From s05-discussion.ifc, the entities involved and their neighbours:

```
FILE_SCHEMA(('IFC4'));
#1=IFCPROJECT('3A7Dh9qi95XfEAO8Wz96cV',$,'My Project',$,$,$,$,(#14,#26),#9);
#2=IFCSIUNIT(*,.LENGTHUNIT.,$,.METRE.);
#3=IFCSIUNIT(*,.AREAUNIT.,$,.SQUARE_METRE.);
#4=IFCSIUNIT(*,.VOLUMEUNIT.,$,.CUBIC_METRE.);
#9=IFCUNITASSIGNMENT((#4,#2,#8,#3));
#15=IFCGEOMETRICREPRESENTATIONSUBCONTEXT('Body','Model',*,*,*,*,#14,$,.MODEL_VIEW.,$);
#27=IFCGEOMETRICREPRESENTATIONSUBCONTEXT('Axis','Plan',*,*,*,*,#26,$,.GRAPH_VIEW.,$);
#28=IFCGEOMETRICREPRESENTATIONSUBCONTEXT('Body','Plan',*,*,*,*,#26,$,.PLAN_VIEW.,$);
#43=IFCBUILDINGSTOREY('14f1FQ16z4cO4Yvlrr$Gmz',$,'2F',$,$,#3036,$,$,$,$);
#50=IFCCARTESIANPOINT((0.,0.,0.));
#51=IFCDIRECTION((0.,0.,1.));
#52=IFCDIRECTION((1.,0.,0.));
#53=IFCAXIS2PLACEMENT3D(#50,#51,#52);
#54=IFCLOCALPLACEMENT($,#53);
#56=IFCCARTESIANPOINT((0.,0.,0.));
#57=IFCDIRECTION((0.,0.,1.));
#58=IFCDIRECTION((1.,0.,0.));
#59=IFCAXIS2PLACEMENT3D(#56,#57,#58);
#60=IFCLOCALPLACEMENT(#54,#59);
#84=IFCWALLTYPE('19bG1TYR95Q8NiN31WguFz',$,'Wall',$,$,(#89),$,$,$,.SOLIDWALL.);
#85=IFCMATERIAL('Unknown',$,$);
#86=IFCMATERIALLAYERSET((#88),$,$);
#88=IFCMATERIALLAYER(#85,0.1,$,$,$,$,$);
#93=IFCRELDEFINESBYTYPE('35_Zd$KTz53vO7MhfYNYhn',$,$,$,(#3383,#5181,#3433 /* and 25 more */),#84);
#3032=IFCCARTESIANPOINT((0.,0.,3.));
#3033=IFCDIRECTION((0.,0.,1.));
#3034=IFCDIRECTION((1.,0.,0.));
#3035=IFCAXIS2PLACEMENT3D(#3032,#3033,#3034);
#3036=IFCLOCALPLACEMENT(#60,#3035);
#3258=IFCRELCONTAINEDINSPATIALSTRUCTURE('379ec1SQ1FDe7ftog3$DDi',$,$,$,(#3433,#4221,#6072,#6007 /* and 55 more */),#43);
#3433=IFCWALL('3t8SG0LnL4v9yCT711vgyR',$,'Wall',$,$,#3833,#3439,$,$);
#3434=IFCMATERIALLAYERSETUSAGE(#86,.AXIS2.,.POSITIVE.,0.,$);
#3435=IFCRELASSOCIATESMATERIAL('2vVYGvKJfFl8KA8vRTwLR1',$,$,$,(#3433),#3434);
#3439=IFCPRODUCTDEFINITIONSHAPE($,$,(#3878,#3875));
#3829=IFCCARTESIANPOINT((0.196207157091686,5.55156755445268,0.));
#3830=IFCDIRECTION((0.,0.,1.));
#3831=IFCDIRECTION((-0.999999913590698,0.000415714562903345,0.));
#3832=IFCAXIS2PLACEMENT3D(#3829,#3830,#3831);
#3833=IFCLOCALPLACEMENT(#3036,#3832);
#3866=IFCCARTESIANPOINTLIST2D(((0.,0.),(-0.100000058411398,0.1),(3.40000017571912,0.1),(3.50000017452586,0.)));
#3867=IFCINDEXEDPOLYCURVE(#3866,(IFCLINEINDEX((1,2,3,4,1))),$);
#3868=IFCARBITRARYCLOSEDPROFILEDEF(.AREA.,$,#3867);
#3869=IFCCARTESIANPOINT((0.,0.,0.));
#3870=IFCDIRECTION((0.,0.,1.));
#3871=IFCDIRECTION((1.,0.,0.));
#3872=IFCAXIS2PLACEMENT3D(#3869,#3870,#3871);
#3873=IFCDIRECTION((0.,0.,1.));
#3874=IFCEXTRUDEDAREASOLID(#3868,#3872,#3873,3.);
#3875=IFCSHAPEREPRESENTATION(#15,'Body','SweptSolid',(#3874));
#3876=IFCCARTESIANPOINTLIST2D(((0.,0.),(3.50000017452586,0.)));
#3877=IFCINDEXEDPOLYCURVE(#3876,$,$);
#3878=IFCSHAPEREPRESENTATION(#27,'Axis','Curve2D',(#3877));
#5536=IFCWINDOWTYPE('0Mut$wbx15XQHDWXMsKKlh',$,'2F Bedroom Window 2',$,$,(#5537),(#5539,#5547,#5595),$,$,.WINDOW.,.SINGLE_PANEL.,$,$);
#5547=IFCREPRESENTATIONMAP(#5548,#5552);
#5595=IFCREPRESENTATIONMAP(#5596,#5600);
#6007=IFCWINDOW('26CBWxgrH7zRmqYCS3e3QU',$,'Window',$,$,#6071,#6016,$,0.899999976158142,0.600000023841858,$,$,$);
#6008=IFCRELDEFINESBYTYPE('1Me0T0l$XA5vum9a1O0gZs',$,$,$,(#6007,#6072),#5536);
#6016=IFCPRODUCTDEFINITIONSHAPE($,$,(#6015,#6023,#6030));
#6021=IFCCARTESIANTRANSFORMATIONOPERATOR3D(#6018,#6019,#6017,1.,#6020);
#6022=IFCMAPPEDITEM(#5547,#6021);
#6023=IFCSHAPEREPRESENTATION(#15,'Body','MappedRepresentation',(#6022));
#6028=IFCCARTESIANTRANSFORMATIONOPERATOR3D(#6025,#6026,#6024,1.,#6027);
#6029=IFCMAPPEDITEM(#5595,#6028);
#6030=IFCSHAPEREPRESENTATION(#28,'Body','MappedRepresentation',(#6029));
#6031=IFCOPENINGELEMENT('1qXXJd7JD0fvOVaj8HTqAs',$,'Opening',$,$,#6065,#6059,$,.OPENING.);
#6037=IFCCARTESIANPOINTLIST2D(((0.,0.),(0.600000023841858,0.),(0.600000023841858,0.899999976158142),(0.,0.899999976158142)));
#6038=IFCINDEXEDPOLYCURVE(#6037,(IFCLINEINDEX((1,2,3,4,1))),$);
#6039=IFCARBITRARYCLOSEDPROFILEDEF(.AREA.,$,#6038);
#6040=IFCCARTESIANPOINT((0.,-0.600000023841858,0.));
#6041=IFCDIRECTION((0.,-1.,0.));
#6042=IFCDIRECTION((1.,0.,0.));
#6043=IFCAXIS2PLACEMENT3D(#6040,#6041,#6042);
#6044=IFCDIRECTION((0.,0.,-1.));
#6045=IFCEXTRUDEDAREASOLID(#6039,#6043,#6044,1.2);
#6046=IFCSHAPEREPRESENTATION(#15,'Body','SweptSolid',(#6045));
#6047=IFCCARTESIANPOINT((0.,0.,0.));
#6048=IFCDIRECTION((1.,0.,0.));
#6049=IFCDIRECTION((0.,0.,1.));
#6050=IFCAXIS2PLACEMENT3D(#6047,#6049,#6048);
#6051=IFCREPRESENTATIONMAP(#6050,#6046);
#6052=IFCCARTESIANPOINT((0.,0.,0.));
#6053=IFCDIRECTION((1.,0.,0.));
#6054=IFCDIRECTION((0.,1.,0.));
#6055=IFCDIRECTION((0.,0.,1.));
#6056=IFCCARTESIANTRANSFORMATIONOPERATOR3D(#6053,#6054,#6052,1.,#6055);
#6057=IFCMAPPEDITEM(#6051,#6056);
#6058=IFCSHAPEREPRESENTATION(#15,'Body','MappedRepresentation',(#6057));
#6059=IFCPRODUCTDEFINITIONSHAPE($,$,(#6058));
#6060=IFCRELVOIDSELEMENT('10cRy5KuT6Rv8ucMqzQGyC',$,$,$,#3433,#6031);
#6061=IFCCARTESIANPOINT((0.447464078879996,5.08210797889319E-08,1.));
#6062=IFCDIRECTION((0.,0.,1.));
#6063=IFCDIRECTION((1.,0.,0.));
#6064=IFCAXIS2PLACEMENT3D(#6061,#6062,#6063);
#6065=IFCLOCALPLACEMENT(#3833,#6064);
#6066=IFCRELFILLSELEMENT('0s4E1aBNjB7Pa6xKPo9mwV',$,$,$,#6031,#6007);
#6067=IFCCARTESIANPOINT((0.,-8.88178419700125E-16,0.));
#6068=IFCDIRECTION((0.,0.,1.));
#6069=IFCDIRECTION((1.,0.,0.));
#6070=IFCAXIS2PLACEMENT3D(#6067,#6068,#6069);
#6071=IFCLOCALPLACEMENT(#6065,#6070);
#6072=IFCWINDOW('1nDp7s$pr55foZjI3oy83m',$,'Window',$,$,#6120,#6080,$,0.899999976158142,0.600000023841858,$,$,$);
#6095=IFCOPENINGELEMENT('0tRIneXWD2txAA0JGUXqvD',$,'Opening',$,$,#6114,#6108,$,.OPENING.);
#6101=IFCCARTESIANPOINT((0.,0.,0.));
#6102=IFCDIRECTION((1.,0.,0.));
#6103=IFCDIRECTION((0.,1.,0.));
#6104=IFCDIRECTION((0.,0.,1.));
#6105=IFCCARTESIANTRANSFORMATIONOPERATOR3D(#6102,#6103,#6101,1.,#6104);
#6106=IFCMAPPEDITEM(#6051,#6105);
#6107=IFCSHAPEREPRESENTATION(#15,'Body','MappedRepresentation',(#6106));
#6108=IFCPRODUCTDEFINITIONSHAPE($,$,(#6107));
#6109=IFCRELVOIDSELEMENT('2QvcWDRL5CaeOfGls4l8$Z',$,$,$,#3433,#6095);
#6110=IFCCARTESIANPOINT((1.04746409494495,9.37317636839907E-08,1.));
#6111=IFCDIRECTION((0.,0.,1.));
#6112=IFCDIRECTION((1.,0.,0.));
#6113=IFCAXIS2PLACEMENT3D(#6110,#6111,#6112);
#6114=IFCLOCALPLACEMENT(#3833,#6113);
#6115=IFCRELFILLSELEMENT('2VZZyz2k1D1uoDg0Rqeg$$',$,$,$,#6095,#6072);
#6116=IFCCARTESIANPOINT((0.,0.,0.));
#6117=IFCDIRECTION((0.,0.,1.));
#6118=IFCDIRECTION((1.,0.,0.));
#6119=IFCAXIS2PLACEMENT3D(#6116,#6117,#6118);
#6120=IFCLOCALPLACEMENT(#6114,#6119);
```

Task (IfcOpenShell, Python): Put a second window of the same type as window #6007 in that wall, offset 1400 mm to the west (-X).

```python
import ifcopenshell
import ifcopenshell.api.feature
import ifcopenshell.api.geometry
import ifcopenshell.api.root
import ifcopenshell.geom
import ifcopenshell.util.element
import ifcopenshell.util.placement
import ifcopenshell.util.shape

model = ifcopenshell.open("s05-discussion.ifc")
settings = ifcopenshell.geom.settings()


def volume(element):
    """Net volume in cubic metres, openings subtracted."""
    shape = ifcopenshell.geom.create_shape(settings, element)
    return ifcopenshell.util.shape.get_volume(shape.geometry)


window = model.by_id(6007)
opening = window.FillsVoids[0].RelatingOpeningElement
wall = opening.VoidsElements[0].RelatingBuildingElement
before = volume(wall)
shift = ifcopenshell.util.placement.get_local_placement(wall.ObjectPlacement)[:3, 0] * 1.4

# copy_class copies the void relationship, type, container and properties, but no geometry.
new_opening = ifcopenshell.api.root.copy_class(model, product=opening)
new_opening.Representation = ifcopenshell.util.element.copy_deep(
    model, opening.Representation, exclude=["IfcGeometricRepresentationContext", "IfcRepresentationMap"]
)
new_window = ifcopenshell.api.root.copy_class(model, product=window)
new_window.Representation = ifcopenshell.util.element.copy_deep(
    model, window.Representation, exclude=["IfcGeometricRepresentationContext", "IfcRepresentationMap"]
)
ifcopenshell.api.feature.add_filling(model, opening=new_opening, element=new_window)

for old, new in ((opening, new_opening), (window, new_window)):
    matrix = ifcopenshell.util.placement.get_local_placement(old.ObjectPlacement)
    matrix[:3, 3] += shift
    ifcopenshell.api.geometry.edit_object_placement(model, product=new, matrix=matrix, is_si=False)

after = volume(wall)

print(f"wall volume {before:.3f} -> {after:.3f} m3")

model.write("s05-discussion_rev.ifc")
```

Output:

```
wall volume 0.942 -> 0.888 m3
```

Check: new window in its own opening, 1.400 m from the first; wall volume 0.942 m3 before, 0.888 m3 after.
